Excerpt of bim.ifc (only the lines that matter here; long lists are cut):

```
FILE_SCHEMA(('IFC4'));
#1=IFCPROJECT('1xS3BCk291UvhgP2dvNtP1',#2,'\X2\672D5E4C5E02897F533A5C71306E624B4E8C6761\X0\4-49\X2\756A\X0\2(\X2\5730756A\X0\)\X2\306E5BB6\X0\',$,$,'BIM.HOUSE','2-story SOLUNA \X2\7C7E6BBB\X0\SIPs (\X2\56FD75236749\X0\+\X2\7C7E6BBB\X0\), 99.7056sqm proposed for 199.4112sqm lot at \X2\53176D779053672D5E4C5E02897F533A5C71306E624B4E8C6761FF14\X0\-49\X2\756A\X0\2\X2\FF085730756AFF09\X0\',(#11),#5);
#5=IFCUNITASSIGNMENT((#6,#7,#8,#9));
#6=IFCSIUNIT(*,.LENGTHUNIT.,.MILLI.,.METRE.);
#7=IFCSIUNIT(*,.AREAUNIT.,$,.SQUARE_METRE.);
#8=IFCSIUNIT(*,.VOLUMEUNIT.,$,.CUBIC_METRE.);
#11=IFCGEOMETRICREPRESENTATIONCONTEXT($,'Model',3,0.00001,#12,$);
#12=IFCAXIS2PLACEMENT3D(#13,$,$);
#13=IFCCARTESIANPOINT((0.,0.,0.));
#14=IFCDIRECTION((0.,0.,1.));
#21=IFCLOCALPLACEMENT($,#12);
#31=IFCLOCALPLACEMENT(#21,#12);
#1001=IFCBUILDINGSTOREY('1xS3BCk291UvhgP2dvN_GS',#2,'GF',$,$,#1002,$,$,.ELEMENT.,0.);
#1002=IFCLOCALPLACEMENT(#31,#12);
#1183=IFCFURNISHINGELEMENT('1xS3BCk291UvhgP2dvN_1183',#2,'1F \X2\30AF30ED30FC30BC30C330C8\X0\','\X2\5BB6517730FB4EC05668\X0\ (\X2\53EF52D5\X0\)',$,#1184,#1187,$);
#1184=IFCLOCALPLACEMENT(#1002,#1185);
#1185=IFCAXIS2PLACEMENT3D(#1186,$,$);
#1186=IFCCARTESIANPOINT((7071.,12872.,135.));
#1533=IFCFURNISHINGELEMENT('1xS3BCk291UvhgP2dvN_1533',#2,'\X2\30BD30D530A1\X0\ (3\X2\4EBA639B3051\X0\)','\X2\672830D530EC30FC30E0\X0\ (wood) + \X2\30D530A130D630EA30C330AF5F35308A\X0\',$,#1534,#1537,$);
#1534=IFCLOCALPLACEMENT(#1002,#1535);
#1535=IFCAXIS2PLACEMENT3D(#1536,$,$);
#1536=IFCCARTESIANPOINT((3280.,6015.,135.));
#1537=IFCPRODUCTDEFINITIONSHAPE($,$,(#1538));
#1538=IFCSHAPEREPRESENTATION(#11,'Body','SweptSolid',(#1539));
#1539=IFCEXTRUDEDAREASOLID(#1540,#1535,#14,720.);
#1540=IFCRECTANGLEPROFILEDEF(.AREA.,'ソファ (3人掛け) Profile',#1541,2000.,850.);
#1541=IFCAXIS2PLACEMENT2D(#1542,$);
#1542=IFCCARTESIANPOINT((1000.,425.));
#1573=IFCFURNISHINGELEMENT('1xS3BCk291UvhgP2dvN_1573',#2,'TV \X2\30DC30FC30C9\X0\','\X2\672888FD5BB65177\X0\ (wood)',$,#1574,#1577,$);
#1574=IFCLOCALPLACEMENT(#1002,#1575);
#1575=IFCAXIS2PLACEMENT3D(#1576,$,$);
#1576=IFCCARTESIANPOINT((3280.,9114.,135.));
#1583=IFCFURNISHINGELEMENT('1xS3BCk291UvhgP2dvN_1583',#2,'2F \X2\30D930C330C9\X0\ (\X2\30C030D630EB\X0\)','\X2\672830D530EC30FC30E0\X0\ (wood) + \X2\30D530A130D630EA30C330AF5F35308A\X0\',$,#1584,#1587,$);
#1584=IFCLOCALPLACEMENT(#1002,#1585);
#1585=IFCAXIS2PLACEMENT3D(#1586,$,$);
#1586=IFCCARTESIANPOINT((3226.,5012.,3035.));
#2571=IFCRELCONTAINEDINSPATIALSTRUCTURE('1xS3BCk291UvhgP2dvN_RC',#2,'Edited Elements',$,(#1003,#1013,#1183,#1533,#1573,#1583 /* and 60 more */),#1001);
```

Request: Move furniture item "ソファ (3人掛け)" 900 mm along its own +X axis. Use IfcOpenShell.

```python
import ifcopenshell
import ifcopenshell.api.geometry
import ifcopenshell.util.placement

model = ifcopenshell.open("bim.ifc")

item = model.by_guid("1xS3BCk291UvhgP2dvN_1533")
matrix = ifcopenshell.util.placement.get_local_placement(item.ObjectPlacement)
matrix[:3, 3] += matrix[:3, 0] * 900.0
ifcopenshell.api.geometry.edit_object_placement(model, product=item, matrix=matrix, is_si=False)

print(ifcopenshell.util.placement.get_local_placement(item.ObjectPlacement).round(3) + 0.0)

model.write("bim_rev.ifc")
```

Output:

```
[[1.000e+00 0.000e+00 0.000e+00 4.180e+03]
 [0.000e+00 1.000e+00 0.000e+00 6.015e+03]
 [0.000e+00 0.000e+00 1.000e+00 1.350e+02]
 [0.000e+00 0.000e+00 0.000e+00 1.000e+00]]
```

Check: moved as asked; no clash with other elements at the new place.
